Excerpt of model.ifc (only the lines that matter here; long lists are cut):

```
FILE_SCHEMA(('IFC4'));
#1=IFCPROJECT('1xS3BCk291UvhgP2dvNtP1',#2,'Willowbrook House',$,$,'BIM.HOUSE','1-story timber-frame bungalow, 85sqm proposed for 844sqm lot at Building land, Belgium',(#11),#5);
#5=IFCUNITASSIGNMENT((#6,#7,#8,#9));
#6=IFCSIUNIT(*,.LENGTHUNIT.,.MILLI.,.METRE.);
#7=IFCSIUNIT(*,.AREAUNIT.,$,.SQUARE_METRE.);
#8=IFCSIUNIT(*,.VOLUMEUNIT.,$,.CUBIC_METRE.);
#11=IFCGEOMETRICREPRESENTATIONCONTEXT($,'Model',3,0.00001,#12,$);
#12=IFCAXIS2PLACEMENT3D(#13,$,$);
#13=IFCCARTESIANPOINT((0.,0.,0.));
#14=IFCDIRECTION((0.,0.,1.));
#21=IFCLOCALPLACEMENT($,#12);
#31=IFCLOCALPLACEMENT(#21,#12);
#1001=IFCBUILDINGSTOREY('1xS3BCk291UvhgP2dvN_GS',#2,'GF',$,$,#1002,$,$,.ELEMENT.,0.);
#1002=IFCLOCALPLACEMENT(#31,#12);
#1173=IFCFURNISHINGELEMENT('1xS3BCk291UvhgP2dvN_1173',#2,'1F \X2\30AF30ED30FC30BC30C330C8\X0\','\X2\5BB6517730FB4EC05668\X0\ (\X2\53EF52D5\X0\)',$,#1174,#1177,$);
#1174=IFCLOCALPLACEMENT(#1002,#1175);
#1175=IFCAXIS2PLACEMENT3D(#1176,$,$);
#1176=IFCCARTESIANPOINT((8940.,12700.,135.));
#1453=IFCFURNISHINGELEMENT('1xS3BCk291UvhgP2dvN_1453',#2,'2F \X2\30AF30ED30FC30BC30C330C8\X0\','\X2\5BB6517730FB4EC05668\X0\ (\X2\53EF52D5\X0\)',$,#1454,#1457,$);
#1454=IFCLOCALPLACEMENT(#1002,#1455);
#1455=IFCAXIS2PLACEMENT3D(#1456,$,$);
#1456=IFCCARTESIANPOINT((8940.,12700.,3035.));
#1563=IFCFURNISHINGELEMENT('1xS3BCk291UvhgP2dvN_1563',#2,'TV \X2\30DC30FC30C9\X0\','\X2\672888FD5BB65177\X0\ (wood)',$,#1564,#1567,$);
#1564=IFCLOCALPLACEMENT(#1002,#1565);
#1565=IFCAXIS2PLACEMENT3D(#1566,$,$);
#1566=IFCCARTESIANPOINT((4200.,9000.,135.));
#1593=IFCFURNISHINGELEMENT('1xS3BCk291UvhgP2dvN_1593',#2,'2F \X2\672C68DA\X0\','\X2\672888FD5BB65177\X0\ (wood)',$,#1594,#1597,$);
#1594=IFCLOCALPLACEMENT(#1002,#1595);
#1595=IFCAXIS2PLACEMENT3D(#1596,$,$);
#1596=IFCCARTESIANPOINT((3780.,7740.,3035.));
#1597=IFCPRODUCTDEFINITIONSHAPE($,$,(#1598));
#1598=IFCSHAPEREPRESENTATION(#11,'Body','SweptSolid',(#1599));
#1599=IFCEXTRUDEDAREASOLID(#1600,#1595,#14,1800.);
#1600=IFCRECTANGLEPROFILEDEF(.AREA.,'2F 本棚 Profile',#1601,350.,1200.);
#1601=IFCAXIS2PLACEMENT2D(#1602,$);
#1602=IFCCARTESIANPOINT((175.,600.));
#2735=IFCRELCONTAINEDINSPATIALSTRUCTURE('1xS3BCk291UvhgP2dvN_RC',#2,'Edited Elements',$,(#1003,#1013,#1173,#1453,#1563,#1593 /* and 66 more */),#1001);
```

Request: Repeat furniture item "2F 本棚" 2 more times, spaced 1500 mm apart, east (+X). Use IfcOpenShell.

```python
import numpy as np
import ifcopenshell
import ifcopenshell.api.geometry
import ifcopenshell.api.root
import ifcopenshell.util.element
import ifcopenshell.util.placement

model = ifcopenshell.open("model.ifc")


def reuse_history(source, copy):
    """copy_class also copies each property set's owner history, people and application; keep the originals."""
    for rel in copy.IsDefinedBy:
        if rel.is_a("IfcRelDefinesByProperties") and (history := rel.RelatingPropertyDefinition.OwnerHistory):
            rel.RelatingPropertyDefinition.OwnerHistory = source.OwnerHistory
            ifcopenshell.util.element.remove_deep2(model, history)


source = model.by_guid("1xS3BCk291UvhgP2dvN_1593")
base = ifcopenshell.util.placement.get_local_placement(source.ObjectPlacement)
step = np.array([1.0, 0.0, 0.0]) * 1500.0

for i in range(1, 3):
    copy = ifcopenshell.api.root.copy_class(model, product=source)
    copy.Representation = ifcopenshell.util.element.copy_deep(
        model, source.Representation, exclude=["IfcGeometricRepresentationContext", "IfcRepresentationMap"]
    )
    reuse_history(source, copy)
    matrix = base.copy()
    matrix[:3, 3] += i * step
    print("added at", matrix[:3, 3].round(3) + 0.0)
    ifcopenshell.api.geometry.edit_object_placement(model, product=copy, matrix=matrix, is_si=False)

model.write("model_updated.ifc")
```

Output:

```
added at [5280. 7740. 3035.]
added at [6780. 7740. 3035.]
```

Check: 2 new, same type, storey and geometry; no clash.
